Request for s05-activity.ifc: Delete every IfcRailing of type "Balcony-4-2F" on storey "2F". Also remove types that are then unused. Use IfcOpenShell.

First a look at what the model holds.

```python
import ifcopenshell
import ifcopenshell.util.element

model = ifcopenshell.open("s05-activity.ifc")
print(model.schema)
storey = next(s for s in model.by_type("IfcBuildingStorey") if s.Name == "2F")
railings = [e for e in ifcopenshell.util.element.get_decomposition(storey) if e.is_a("IfcRailing")]
seen = {}
for e in railings:
    element_type = ifcopenshell.util.element.get_type(e)
    name = element_type.Name if element_type not in (None, e) else None
    seen[name] = seen.get(name, 0) + 1
for name, count in sorted(seen.items(), key=str):
    print(count, "x", name)
```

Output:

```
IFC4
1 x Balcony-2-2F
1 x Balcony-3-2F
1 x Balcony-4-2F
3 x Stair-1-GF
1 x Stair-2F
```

```python
import ifcopenshell
import ifcopenshell.api.root
import ifcopenshell.util.element

model = ifcopenshell.open("s05-activity.ifc")

storey = next(s for s in model.by_type("IfcBuildingStorey") if s.Name == "2F")
railings = [e for e in ifcopenshell.util.element.get_decomposition(storey) if e.is_a("IfcRailing")]
targets = [e for e in railings if (t := ifcopenshell.util.element.get_type(e)) not in (None, e) and t.Name == "Balcony-4-2F"]
types = {ifcopenshell.util.element.get_type(e) for e in targets} - {None, *targets}

for e in targets:
    ifcopenshell.api.root.remove_product(model, product=e)
print(len(targets), "removed")

unused = [t for t in types if not ifcopenshell.util.element.get_types(t)]
for t in unused:
    ifcopenshell.api.root.remove_product(model, product=t)
print(len(unused), "unused types removed")

model.write("s05-activity_updated.ifc")
```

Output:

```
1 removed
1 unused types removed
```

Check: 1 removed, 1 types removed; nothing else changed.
